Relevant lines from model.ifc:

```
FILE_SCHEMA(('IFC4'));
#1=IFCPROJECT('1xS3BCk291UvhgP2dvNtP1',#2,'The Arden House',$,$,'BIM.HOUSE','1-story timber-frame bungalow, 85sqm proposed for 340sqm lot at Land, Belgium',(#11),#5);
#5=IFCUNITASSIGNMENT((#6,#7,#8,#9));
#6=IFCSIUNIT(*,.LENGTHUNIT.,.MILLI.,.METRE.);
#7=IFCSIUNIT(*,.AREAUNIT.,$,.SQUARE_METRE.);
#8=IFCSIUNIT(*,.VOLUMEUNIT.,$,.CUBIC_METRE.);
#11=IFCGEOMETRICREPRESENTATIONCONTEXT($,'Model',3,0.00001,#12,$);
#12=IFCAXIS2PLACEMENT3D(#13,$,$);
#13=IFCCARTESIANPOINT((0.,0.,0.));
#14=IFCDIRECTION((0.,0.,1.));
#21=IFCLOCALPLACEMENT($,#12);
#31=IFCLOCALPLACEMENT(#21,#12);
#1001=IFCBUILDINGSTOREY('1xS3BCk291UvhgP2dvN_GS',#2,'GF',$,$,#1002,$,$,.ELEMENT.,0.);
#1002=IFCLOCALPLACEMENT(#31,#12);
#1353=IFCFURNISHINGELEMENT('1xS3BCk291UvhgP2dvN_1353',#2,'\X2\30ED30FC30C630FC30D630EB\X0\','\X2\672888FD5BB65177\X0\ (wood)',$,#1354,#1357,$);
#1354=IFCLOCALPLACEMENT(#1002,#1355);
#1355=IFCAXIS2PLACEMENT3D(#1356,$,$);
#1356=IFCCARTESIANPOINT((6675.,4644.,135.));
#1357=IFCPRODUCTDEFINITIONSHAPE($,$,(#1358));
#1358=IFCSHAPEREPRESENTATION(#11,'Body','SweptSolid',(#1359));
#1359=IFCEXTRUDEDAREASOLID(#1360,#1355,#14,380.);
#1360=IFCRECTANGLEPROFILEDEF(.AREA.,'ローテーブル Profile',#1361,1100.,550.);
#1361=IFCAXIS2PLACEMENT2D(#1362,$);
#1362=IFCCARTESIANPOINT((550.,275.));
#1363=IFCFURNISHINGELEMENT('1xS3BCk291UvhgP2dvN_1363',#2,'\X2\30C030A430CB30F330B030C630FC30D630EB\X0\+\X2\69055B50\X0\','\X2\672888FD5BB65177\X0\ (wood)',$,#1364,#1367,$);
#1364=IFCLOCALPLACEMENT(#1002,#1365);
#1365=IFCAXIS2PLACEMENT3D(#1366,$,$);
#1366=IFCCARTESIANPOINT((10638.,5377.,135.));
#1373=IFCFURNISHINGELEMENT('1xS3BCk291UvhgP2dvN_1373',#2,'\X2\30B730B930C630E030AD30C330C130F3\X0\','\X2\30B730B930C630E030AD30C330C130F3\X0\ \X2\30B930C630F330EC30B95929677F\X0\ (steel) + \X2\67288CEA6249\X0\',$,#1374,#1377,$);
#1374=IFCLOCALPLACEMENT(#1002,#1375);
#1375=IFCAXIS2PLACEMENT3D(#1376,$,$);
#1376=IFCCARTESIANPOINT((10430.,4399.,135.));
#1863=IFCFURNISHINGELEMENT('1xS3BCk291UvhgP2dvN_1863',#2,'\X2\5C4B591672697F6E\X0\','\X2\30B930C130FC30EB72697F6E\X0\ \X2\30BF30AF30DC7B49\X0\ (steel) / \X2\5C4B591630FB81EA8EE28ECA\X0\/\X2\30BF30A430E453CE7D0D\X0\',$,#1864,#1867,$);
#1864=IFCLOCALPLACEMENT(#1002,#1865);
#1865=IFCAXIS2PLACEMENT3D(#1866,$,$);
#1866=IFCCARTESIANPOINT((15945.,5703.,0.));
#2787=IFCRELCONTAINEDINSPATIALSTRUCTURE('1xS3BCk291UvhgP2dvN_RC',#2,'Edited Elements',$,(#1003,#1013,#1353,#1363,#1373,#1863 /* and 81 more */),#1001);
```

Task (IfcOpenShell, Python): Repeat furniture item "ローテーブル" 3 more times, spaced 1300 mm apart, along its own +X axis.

```python
import ifcopenshell
import ifcopenshell.api.geometry
import ifcopenshell.api.root
import ifcopenshell.util.element
import ifcopenshell.util.placement

model = ifcopenshell.open("model.ifc")


def reuse_history(source, copy):
    """copy_class also copies each property set's owner history, people and application; keep the originals."""
    for rel in copy.IsDefinedBy:
        if rel.is_a("IfcRelDefinesByProperties") and (history := rel.RelatingPropertyDefinition.OwnerHistory):
            rel.RelatingPropertyDefinition.OwnerHistory = source.OwnerHistory
            ifcopenshell.util.element.remove_deep2(model, history)


source = model.by_id(1353)
base = ifcopenshell.util.placement.get_local_placement(source.ObjectPlacement)
step = base[:3, 0] * 1300.0

for i in range(1, 4):
    copy = ifcopenshell.api.root.copy_class(model, product=source)
    copy.Representation = ifcopenshell.util.element.copy_deep(
        model, source.Representation, exclude=["IfcGeometricRepresentationContext", "IfcRepresentationMap"]
    )
    reuse_history(source, copy)
    matrix = base.copy()
    matrix[:3, 3] += i * step
    print("added at", matrix[:3, 3].round(3) + 0.0)
    ifcopenshell.api.geometry.edit_object_placement(model, product=copy, matrix=matrix, is_si=False)

model.write("model_edited.ifc")
```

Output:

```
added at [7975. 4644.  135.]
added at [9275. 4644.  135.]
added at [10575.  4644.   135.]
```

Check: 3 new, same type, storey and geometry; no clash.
